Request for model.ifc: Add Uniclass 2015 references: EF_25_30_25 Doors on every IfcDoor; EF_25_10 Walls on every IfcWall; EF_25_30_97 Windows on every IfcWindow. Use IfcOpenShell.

First a look at what the model holds.

```python
import ifcopenshell

model = ifcopenshell.open("model.ifc")
print(model.schema)
print("classifications:", [c.Name for c in model.by_type("IfcClassification")])
for ifc_class in ("IfcDoor", "IfcRoof", "IfcStair", "IfcWall", "IfcWindow"):
    print(ifc_class, len(model.by_type(ifc_class)))
```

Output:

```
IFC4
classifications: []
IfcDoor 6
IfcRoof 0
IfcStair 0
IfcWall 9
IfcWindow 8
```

```python
import ifcopenshell
import ifcopenshell.api.classification

model = ifcopenshell.open("model.ifc")

system = ifcopenshell.api.classification.add_classification(model, classification="Uniclass 2015")

codes = {
    "IfcDoor": ("EF_25_30_25", "Doors"),
    "IfcWall": ("EF_25_10", "Walls"),
    "IfcWindow": ("EF_25_30_97", "Windows"),
}
for ifc_class, (code, name) in codes.items():
    products = model.by_type(ifc_class)
    ifcopenshell.api.classification.add_reference(
        model, products=products, classification=system, identification=code, name=name
    )
    print(code, len(products))

model.write("model_edited.ifc")
```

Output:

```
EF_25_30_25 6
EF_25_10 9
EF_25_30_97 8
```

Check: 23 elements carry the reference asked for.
